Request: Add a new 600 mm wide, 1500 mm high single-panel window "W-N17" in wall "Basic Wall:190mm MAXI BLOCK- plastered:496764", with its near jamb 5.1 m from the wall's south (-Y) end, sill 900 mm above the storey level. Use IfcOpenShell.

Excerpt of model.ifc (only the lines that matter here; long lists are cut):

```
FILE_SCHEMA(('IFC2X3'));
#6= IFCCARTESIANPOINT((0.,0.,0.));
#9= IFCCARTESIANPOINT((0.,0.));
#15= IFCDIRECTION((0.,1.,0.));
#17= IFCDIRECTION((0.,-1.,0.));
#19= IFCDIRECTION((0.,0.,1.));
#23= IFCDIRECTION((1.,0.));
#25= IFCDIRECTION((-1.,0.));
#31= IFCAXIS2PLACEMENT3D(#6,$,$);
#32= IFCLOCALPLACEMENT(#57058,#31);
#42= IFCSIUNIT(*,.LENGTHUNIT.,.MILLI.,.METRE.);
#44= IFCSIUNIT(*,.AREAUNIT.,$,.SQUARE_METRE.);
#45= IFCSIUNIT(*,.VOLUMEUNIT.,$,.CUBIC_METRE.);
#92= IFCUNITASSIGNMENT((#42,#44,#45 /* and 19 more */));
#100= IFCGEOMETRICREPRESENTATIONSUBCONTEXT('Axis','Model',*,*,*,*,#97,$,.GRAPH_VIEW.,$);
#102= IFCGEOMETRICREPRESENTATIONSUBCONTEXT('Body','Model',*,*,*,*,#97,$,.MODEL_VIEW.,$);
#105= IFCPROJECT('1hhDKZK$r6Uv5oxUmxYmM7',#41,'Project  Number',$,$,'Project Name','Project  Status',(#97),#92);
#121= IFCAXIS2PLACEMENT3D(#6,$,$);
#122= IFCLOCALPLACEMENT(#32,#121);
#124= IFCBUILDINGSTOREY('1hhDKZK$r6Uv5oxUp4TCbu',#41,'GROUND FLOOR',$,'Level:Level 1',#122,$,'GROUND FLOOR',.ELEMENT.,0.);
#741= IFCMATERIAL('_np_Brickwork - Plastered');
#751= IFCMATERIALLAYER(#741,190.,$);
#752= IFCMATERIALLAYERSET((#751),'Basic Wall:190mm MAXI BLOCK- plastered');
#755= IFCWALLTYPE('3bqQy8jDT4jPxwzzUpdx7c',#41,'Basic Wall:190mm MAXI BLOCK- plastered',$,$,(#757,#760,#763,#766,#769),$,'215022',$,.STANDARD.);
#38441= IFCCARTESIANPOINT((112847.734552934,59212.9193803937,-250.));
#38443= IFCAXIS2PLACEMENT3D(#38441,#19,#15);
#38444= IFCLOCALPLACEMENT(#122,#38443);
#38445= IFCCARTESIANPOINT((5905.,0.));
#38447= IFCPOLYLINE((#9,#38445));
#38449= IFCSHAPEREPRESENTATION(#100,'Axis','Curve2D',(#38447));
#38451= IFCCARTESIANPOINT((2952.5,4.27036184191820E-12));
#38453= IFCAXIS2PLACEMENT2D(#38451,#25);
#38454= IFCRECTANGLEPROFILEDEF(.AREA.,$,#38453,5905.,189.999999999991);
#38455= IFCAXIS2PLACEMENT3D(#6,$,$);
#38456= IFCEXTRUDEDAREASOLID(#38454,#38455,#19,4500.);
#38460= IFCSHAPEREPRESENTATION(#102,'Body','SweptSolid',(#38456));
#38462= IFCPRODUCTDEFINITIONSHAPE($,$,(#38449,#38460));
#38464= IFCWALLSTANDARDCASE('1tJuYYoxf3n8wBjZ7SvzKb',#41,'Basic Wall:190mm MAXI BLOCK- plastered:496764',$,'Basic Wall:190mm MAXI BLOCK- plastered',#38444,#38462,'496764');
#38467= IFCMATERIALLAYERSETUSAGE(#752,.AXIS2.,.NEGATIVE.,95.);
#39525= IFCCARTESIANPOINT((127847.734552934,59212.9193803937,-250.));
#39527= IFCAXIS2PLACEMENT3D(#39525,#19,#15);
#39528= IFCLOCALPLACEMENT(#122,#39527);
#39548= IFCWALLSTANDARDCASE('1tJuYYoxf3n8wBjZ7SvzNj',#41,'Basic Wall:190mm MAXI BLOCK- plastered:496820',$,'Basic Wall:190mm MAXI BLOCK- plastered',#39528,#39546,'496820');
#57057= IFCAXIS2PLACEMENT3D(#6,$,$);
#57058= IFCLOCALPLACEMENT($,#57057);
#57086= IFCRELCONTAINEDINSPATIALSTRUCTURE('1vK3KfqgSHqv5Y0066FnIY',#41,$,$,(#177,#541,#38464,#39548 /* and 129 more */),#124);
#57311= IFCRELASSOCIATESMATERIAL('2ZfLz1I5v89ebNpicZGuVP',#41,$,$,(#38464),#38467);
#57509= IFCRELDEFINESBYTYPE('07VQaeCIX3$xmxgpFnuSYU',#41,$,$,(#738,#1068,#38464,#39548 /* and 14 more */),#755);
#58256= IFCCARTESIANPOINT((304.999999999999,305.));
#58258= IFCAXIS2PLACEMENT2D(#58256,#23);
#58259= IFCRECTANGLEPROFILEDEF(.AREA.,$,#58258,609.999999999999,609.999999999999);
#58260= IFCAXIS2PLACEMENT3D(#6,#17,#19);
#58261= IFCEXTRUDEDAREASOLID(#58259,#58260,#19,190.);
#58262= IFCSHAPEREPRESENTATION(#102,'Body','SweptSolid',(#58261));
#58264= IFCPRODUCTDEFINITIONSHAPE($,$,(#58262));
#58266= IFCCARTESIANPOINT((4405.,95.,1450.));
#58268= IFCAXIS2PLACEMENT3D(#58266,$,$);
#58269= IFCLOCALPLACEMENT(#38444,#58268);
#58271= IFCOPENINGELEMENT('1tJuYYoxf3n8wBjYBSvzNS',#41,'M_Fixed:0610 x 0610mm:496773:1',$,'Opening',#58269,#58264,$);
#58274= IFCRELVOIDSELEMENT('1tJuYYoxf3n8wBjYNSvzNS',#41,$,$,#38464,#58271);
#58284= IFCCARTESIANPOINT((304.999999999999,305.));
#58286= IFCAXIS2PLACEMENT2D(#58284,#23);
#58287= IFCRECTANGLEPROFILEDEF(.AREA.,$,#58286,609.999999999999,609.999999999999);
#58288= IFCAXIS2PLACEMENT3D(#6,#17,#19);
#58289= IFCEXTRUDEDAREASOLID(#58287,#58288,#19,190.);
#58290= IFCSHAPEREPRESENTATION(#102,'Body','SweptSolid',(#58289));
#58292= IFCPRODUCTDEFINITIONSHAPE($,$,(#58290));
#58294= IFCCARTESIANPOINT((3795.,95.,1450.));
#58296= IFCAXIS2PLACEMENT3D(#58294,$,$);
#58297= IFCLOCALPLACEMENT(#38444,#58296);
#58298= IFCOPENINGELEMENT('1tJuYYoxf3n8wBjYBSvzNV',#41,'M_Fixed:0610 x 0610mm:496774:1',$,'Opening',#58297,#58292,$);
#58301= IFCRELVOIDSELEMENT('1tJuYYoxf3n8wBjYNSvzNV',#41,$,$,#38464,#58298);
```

```python
import numpy as np
import ifcopenshell
import ifcopenshell.api.feature
import ifcopenshell.api.geometry
import ifcopenshell.api.root
import ifcopenshell.api.spatial
import ifcopenshell.api.type
import ifcopenshell.geom
import ifcopenshell.util.element
import ifcopenshell.util.placement
import ifcopenshell.util.representation
import ifcopenshell.util.shape
import ifcopenshell.util.unit

model = ifcopenshell.open("model.ifc")
unit_scale = ifcopenshell.util.unit.calculate_unit_scale(model)
settings = ifcopenshell.geom.settings()


def volume(element):
    """Net volume in cubic metres, openings subtracted."""
    shape = ifcopenshell.geom.create_shape(settings, element)
    return ifcopenshell.util.shape.get_volume(shape.geometry)


wall = model.by_guid("1tJuYYoxf3n8wBjZ7SvzKb")
storey = ifcopenshell.util.element.get_container(wall, ifc_class="IfcBuildingStorey")
context = ifcopenshell.util.representation.get_context(model, "Model", "Body", "MODEL_VIEW")
before = volume(wall)

width, height, from_end, sill = 0.6, 1.5, 5.1, 0.9  # metres

# The wall runs along its own X axis, and the end named is its -X end.
wall_shape = ifcopenshell.geom.create_shape(settings, wall)
x, y, z = ifcopenshell.util.shape.get_vertices(wall_shape.geometry).T
start = x.min() + from_end
face, thickness = float(y.min()), float(y.max() - y.min())
wall_matrix = ifcopenshell.util.placement.get_local_placement(wall.ObjectPlacement)
level = ifcopenshell.util.placement.get_local_placement(storey.ObjectPlacement)[2, 3]


def in_wall(x, y):
    """Placement at x, y metres in the wall's axes, at sill height."""
    matrix = wall_matrix.copy()
    matrix[:, 3] = wall_matrix @ np.array([x / unit_scale, y / unit_scale, 0.0, 1.0])
    matrix[2, 3] = level + sill / unit_scale
    return matrix


# Opening: a box that overshoots both wall faces by 50 mm.
opening = ifcopenshell.api.root.create_entity(model, ifc_class="IfcOpeningElement")
box = ifcopenshell.api.geometry.add_wall_representation(
    model, context=context, length=width, height=height, thickness=thickness + 0.1
)
ifcopenshell.api.geometry.assign_representation(model, product=opening, representation=box)
ifcopenshell.api.geometry.edit_object_placement(model, product=opening, matrix=in_wall(start, face - 0.05), is_si=False)
ifcopenshell.api.feature.add_feature(model, feature=opening, element=wall)

window = ifcopenshell.api.root.create_entity(model, ifc_class="IfcWindow", name="W-N17")
window.OverallWidth, window.OverallHeight = width / unit_scale, height / unit_scale
body = ifcopenshell.api.geometry.add_window_representation(
    model,
    context=context,
    overall_width=window.OverallWidth,
    overall_height=window.OverallHeight,
    partition_type="SINGLE_PANEL",
)
ifcopenshell.api.geometry.assign_representation(model, product=window, representation=body)
ifcopenshell.api.spatial.assign_container(model, products=[window], relating_structure=storey)
fills = ifcopenshell.api.feature.add_filling(model, opening=opening, element=window)
fills.OwnerHistory = window.OwnerHistory  # required in IFC2X3

# IFC2X3 keeps the operation on the window style.
style = ifcopenshell.api.root.create_entity(model, ifc_class="IfcWindowStyle", name="W-N17")
style.OperationType, style.ConstructionType = "SINGLE_PANEL", "NOTDEFINED"
style.ParameterTakesPrecedence = style.Sizeable = False
ifcopenshell.api.type.assign_type(model, related_objects=[window], relating_type=style)

# Centre the window in the wall's thickness.
ifcopenshell.api.geometry.edit_object_placement(model, product=window, matrix=in_wall(start, face), is_si=False)
window_shape = ifcopenshell.geom.create_shape(settings, window)
depth = ifcopenshell.util.shape.get_vertices(window_shape.geometry)[:, 1]
offset = face + thickness / 2 - (depth.min() + depth.max()) / 2
ifcopenshell.api.geometry.edit_object_placement(model, product=window, matrix=in_wall(start, offset), is_si=False)

after = volume(wall)

print(f"wall volume {before:.3f} -> {after:.3f} m3")

model.write("model_rev.ifc")
```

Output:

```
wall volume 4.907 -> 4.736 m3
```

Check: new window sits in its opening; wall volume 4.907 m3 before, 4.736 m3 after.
